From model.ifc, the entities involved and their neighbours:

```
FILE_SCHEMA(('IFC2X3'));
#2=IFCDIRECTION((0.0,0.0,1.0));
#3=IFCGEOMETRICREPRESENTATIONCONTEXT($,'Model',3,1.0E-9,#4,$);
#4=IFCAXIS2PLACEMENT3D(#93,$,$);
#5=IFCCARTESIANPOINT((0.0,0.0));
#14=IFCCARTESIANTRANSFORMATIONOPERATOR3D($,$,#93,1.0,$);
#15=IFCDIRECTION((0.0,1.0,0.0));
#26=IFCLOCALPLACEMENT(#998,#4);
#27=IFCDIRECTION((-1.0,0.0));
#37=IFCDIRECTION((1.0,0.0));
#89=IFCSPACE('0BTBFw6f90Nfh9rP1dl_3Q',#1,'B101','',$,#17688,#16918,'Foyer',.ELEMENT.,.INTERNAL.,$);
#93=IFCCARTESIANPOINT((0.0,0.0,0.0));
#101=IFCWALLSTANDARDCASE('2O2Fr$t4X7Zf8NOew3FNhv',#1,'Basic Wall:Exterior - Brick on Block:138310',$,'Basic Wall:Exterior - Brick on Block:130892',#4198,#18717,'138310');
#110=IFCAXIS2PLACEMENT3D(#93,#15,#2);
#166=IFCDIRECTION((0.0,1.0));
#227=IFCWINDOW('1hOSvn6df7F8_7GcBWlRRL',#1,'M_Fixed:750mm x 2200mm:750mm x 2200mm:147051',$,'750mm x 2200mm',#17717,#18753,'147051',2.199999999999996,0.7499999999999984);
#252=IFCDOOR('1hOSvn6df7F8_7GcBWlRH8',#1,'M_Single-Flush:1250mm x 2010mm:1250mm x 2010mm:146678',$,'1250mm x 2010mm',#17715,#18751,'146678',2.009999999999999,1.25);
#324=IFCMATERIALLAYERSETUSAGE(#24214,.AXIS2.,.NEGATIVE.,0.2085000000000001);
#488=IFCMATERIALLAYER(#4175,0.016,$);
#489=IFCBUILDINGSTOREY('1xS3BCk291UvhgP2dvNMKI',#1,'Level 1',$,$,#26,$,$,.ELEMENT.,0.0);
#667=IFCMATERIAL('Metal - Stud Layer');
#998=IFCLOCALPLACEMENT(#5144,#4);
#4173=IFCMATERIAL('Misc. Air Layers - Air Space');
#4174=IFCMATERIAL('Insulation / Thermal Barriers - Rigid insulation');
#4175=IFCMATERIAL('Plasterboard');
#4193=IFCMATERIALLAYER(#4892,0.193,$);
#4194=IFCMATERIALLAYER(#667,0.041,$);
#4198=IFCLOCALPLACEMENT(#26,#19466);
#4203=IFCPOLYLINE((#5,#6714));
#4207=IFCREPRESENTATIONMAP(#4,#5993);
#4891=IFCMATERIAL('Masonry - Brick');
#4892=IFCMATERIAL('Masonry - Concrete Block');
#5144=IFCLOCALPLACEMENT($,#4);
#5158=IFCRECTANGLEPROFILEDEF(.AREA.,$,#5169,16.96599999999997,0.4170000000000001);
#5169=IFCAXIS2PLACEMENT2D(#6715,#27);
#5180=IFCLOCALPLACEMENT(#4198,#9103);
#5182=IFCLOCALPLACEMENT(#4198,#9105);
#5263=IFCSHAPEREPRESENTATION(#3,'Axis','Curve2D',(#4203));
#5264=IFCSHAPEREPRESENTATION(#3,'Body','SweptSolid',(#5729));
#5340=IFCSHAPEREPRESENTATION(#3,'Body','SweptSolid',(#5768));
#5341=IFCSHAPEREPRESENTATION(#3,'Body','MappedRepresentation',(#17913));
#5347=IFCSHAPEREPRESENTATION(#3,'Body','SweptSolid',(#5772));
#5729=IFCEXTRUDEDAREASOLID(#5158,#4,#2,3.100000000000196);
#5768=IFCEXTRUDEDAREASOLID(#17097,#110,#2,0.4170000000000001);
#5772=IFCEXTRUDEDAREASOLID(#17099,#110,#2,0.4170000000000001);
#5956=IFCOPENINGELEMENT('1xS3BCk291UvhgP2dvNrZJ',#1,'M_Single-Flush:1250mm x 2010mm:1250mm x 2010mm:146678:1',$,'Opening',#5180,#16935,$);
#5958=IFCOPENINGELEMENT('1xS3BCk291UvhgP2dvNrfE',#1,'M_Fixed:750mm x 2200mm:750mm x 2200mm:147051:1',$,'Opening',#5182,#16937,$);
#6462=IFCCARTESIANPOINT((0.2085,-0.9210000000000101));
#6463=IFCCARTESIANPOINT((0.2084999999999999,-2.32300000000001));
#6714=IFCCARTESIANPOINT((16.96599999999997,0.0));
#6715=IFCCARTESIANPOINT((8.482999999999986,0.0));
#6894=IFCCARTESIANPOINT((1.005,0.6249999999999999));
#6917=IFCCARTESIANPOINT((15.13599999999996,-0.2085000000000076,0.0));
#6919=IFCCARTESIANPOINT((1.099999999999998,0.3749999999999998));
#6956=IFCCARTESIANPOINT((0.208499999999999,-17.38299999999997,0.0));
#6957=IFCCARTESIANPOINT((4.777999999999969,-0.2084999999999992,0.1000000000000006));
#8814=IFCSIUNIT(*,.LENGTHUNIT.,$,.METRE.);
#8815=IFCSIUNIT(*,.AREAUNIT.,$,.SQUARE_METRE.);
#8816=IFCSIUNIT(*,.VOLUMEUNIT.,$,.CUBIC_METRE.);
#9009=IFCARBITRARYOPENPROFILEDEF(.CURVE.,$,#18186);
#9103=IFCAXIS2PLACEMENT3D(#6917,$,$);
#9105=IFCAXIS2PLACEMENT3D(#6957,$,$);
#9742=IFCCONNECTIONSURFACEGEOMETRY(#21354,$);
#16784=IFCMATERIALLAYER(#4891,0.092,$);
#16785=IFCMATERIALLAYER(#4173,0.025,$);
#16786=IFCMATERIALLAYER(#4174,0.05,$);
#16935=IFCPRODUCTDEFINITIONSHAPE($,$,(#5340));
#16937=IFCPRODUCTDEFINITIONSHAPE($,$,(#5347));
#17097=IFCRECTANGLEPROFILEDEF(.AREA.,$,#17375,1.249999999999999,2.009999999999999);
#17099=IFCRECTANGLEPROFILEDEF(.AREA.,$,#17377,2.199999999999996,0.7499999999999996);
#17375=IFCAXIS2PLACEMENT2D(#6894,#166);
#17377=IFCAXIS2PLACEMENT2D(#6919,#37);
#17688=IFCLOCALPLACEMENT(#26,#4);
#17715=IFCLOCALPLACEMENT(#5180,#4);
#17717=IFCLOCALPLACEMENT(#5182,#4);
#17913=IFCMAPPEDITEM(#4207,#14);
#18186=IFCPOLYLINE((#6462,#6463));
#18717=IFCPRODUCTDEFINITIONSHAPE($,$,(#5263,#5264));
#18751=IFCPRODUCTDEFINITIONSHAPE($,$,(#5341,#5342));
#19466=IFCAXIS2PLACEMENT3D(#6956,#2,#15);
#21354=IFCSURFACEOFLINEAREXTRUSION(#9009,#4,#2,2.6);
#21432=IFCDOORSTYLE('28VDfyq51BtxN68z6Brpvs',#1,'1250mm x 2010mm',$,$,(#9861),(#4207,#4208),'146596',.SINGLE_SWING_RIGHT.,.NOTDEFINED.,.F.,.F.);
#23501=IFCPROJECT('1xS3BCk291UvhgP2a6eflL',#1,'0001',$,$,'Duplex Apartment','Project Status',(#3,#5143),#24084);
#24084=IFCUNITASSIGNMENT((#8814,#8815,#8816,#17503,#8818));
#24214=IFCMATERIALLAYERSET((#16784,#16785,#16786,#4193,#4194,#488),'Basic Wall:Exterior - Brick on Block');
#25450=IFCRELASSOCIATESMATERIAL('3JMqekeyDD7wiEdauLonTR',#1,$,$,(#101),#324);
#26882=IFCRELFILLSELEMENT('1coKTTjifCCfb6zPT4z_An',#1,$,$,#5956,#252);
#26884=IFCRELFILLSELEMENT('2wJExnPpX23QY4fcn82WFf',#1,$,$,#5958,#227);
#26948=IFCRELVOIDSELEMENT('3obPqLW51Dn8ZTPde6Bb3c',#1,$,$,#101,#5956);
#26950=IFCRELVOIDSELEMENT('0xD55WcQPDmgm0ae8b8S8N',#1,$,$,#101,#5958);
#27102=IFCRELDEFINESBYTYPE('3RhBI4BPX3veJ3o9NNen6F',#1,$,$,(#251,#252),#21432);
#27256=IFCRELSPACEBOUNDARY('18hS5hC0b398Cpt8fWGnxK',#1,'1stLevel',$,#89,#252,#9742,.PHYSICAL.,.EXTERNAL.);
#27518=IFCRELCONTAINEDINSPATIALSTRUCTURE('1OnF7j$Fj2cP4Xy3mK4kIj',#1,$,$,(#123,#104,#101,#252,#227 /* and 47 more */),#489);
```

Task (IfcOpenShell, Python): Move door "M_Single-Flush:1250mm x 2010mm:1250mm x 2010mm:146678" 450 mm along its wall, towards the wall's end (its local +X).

```python
import numpy as np
import ifcopenshell
import ifcopenshell.api.geometry
import ifcopenshell.util.placement
import ifcopenshell.util.unit

model = ifcopenshell.open("model.ifc")
unit_scale = ifcopenshell.util.unit.calculate_unit_scale(model)

door = model.by_id(252)
opening = door.FillsVoids[0].RelatingOpeningElement
wall = opening.VoidsElements[0].RelatingBuildingElement

wall_matrix = ifcopenshell.util.placement.get_local_placement(wall.ObjectPlacement)
shift = wall_matrix[:3, 0] * 0.45 / unit_scale
before = ifcopenshell.util.placement.get_local_placement(door.ObjectPlacement)[:3, 3].copy()

# The door is placed relative to its opening, so it follows when the opening moves.
matrix = ifcopenshell.util.placement.get_local_placement(opening.ObjectPlacement)
matrix[:3, 3] += shift
ifcopenshell.api.geometry.edit_object_placement(
    model, product=opening, matrix=matrix, is_si=False, should_transform_children=True
)

# Space boundary surfaces are stored in each space's coordinates; move them too.
for rel in door.ProvidesBoundaries:
    if not rel.ConnectionGeometry:
        continue
    surface = rel.ConnectionGeometry.SurfaceOnRelatingElement
    space_matrix = ifcopenshell.util.placement.get_local_placement(rel.RelatingSpace.ObjectPlacement)
    point = np.array(surface.Position.Location.Coordinates) + space_matrix[:3, :3].T @ shift
    surface.Position = model.createIfcAxis2Placement3D(
        model.createIfcCartesianPoint(point.tolist()), surface.Position.Axis, surface.Position.RefDirection
    )

after = ifcopenshell.util.placement.get_local_placement(door.ObjectPlacement)[:3, 3]
print("door moved by", (after - before).round(3) + 0.0)

model.write("model_v2.ifc")
```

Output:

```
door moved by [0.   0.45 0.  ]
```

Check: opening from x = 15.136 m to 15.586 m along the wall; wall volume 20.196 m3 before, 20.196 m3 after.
